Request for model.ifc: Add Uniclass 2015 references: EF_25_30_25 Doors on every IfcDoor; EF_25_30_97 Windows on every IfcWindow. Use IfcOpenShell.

First a look at what the model holds.

```python
import ifcopenshell

model = ifcopenshell.open("model.ifc")
print(model.schema)
print("classifications:", [c.Name for c in model.by_type("IfcClassification")])
for ifc_class in ("IfcDoor", "IfcRoof", "IfcStair", "IfcWall", "IfcWindow"):
    print(ifc_class, len(model.by_type(ifc_class)))
```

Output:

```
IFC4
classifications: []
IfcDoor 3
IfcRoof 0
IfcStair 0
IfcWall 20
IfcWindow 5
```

```python
import ifcopenshell
import ifcopenshell.api.classification

model = ifcopenshell.open("model.ifc")

system = ifcopenshell.api.classification.add_classification(model, classification="Uniclass 2015")

codes = {
    "IfcDoor": ("EF_25_30_25", "Doors"),
    "IfcWindow": ("EF_25_30_97", "Windows"),
}
for ifc_class, (code, name) in codes.items():
    products = model.by_type(ifc_class)
    ifcopenshell.api.classification.add_reference(
        model, products=products, classification=system, identification=code, name=name
    )
    print(code, len(products))

model.write("model_updated.ifc")
```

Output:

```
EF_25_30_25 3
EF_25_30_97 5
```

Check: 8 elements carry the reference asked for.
